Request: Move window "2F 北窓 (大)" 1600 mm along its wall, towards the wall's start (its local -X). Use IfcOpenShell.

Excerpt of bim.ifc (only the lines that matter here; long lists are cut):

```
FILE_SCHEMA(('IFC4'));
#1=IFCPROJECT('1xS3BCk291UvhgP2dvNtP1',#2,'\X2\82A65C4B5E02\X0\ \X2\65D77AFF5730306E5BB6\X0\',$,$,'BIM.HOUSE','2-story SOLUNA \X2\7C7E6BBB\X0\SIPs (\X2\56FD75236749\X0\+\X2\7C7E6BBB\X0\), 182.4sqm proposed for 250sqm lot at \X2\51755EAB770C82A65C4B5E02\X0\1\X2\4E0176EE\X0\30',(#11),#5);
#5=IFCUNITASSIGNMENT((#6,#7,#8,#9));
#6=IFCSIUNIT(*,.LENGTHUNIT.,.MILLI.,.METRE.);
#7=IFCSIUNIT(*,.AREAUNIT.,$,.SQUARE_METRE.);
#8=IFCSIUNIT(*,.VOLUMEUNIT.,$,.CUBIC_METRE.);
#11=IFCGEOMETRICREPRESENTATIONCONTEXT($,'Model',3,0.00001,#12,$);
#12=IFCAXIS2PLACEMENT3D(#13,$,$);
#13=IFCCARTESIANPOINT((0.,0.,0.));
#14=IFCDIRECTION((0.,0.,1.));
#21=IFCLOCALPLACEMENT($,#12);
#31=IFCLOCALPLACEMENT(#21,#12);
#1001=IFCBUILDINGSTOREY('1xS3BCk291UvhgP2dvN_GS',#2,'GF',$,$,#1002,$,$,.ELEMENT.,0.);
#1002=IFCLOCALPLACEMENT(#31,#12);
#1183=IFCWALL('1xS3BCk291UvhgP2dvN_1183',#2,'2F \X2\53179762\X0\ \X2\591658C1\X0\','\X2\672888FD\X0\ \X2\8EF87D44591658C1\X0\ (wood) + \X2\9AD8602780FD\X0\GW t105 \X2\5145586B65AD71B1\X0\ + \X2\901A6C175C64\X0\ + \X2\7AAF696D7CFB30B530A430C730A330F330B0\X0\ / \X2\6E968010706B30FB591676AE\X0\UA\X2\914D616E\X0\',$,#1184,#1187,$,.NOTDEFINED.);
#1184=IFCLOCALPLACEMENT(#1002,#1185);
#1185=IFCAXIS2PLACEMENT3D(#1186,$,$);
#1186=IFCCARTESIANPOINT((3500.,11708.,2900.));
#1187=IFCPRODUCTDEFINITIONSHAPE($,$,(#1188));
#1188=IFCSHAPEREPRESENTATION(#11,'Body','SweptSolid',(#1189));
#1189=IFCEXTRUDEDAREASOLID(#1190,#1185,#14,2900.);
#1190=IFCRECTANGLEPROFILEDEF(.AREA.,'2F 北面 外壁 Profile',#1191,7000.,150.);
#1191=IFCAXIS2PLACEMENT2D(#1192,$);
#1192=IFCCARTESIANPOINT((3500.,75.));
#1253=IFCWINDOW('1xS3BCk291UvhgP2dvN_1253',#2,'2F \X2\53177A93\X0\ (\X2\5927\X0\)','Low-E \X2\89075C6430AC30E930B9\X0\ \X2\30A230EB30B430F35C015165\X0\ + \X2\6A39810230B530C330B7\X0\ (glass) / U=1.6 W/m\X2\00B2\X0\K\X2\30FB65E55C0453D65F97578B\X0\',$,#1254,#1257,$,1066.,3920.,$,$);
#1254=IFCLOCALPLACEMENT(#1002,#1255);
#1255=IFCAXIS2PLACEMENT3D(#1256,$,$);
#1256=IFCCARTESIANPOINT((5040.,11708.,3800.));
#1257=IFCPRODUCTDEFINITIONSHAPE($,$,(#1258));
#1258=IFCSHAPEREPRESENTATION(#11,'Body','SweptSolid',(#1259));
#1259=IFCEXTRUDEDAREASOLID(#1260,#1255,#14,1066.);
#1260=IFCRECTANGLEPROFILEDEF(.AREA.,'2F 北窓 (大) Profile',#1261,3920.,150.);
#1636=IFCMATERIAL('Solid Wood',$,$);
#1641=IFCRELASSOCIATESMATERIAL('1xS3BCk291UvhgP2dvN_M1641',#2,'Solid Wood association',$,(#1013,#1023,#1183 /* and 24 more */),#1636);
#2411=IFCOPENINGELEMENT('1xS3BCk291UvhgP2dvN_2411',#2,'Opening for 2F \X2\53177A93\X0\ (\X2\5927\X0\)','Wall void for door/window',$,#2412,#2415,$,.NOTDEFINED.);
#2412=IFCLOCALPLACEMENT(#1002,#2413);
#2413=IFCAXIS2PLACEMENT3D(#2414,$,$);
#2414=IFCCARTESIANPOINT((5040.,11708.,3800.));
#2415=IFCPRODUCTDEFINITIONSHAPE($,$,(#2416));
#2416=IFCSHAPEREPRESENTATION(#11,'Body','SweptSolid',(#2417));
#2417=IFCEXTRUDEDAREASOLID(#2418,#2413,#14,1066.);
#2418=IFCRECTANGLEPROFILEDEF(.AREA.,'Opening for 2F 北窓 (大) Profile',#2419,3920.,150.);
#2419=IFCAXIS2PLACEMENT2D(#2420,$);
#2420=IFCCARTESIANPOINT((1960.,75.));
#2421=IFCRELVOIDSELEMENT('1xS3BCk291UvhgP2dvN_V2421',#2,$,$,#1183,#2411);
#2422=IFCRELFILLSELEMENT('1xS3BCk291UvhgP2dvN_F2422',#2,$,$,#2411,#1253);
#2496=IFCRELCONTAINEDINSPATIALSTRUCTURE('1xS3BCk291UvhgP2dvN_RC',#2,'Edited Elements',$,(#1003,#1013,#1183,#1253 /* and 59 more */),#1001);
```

```python
import ifcopenshell
import ifcopenshell.api.geometry
import ifcopenshell.util.placement
import ifcopenshell.util.unit

model = ifcopenshell.open("bim.ifc")
unit_scale = ifcopenshell.util.unit.calculate_unit_scale(model)

window = model.by_guid("1xS3BCk291UvhgP2dvN_1253")
opening = window.FillsVoids[0].RelatingOpeningElement
wall = opening.VoidsElements[0].RelatingBuildingElement

wall_matrix = ifcopenshell.util.placement.get_local_placement(wall.ObjectPlacement)
shift = wall_matrix[:3, 0] * -1.6 / unit_scale
before = ifcopenshell.util.placement.get_local_placement(window.ObjectPlacement)[:3, 3].copy()

# The window is not placed relative to its opening, so move both.
for product in (opening, window):
    matrix = ifcopenshell.util.placement.get_local_placement(product.ObjectPlacement)
    matrix[:3, 3] += shift
    ifcopenshell.api.geometry.edit_object_placement(model, product=product, matrix=matrix, is_si=False)

after = ifcopenshell.util.placement.get_local_placement(window.ObjectPlacement)[:3, 3]
print("window moved by", (after - before).round(3) + 0.0)

model.write("bim_v2.ifc")
```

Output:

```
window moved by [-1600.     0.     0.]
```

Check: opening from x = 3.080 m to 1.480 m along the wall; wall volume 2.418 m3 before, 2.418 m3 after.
